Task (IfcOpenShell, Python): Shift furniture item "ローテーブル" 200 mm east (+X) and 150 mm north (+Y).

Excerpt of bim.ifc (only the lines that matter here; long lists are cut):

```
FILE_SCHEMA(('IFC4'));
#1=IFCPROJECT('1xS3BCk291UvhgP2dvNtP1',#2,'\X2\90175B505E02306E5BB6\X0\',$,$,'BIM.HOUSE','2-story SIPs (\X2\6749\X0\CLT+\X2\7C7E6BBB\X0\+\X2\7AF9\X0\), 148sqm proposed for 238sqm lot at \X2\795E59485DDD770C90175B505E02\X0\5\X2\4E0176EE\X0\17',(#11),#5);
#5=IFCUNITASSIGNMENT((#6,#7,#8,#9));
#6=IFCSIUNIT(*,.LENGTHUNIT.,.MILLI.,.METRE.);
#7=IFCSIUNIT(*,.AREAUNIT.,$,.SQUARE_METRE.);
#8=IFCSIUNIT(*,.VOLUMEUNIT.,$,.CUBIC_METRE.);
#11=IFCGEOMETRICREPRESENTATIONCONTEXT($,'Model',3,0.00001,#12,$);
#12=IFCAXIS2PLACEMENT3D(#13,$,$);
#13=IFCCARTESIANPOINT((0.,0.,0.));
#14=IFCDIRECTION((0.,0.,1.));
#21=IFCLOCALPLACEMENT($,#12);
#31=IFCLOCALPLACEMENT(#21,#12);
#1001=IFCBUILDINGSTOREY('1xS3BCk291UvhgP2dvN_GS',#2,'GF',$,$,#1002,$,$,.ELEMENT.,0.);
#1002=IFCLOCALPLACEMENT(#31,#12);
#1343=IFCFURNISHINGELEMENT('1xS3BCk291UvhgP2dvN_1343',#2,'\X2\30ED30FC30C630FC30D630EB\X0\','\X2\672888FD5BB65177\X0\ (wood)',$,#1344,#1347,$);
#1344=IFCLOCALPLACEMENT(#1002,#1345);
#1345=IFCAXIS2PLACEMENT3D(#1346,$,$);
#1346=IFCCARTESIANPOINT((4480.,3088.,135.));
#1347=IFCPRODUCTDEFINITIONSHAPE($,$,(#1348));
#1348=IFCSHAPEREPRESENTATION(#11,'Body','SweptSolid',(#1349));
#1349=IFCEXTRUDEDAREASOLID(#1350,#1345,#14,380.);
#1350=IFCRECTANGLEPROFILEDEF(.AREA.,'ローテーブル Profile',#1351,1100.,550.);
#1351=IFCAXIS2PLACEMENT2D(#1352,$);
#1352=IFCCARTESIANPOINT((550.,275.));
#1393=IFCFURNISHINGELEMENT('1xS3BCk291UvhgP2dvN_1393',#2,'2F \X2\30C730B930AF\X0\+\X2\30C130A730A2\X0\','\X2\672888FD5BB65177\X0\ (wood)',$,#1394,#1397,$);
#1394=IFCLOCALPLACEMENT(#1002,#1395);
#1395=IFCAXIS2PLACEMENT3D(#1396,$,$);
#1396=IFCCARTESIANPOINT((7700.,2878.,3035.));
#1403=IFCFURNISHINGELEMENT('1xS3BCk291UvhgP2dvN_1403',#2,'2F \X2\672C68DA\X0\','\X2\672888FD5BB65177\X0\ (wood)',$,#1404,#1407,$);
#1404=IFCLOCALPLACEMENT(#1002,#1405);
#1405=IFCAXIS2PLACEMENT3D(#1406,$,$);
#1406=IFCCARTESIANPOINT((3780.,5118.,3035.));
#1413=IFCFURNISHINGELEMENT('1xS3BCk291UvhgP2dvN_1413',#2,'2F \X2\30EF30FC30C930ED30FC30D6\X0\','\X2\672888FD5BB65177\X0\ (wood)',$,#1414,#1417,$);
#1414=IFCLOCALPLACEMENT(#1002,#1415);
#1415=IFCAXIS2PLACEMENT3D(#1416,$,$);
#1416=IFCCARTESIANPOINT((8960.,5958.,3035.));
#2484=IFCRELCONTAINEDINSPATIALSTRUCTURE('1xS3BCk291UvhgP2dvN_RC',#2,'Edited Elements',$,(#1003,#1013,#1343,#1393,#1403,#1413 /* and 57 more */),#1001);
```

```python
import ifcopenshell
import ifcopenshell.api.geometry
import ifcopenshell.util.placement

model = ifcopenshell.open("bim.ifc")

item = model.by_id(1343)
matrix = ifcopenshell.util.placement.get_local_placement(item.ObjectPlacement)
matrix[0, 3] += 200.0
matrix[1, 3] += 150.0
ifcopenshell.api.geometry.edit_object_placement(model, product=item, matrix=matrix, is_si=False)

print(ifcopenshell.util.placement.get_local_placement(item.ObjectPlacement).round(3) + 0.0)

model.write("bim-out.ifc")
```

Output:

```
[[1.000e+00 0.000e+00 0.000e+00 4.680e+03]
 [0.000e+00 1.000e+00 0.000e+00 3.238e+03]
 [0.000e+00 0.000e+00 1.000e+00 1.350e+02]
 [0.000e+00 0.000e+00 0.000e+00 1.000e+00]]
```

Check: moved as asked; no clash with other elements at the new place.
